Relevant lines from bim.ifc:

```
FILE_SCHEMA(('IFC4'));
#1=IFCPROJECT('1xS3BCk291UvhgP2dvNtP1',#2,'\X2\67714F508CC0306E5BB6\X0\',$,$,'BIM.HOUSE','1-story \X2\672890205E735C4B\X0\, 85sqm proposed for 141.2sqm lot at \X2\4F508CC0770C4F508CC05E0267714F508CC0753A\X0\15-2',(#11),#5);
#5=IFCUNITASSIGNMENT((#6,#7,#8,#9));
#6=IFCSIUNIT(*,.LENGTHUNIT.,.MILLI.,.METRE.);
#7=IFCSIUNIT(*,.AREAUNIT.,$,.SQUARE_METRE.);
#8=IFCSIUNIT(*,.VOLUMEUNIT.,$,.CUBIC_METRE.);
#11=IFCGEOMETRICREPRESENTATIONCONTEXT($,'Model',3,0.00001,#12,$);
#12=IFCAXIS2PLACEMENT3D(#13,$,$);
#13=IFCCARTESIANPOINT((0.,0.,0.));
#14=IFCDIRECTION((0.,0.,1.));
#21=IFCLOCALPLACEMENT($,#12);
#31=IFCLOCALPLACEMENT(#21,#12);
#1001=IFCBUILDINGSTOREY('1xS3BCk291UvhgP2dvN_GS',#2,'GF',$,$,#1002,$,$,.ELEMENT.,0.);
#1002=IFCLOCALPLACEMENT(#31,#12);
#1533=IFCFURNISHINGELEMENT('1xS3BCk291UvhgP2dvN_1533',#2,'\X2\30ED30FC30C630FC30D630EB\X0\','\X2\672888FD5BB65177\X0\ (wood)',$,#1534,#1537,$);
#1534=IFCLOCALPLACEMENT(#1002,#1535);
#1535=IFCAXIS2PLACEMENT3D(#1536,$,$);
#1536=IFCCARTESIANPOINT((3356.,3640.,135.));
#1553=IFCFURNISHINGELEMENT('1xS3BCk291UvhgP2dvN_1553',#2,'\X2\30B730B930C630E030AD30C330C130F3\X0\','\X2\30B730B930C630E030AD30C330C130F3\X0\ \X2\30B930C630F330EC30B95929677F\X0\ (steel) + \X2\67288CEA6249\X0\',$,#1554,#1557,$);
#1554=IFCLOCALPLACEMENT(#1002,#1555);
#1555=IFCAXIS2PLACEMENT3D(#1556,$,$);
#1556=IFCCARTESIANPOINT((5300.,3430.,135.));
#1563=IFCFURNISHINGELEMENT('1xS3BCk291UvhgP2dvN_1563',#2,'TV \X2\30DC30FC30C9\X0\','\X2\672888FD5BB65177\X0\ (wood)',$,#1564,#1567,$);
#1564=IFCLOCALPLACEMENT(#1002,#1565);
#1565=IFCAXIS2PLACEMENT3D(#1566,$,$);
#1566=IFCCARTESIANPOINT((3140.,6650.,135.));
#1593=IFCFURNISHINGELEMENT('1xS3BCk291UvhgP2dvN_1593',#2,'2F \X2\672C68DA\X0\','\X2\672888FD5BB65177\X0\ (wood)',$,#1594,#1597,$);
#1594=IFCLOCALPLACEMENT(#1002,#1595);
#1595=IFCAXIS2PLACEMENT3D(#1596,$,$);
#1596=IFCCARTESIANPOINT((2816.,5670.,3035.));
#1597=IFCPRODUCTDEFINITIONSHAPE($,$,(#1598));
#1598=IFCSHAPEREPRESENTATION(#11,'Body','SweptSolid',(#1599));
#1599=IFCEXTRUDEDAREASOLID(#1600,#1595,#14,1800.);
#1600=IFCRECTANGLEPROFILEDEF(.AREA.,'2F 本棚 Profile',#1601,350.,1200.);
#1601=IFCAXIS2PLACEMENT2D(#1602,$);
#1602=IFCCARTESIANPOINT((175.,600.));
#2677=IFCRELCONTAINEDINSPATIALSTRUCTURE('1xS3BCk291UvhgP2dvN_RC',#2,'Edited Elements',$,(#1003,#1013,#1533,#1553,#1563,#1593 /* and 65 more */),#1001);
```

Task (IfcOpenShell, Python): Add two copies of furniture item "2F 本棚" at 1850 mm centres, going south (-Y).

```python
import numpy as np
import ifcopenshell
import ifcopenshell.api.geometry
import ifcopenshell.api.root
import ifcopenshell.util.element
import ifcopenshell.util.placement

model = ifcopenshell.open("bim.ifc")


def reuse_history(source, copy):
    """copy_class also copies each property set's owner history, people and application; keep the originals."""
    for rel in copy.IsDefinedBy:
        if rel.is_a("IfcRelDefinesByProperties") and (history := rel.RelatingPropertyDefinition.OwnerHistory):
            rel.RelatingPropertyDefinition.OwnerHistory = source.OwnerHistory
            ifcopenshell.util.element.remove_deep2(model, history)


source = model.by_guid("1xS3BCk291UvhgP2dvN_1593")
base = ifcopenshell.util.placement.get_local_placement(source.ObjectPlacement)
step = np.array([0.0, -1.0, 0.0]) * 1850.0

for i in range(1, 3):
    copy = ifcopenshell.api.root.copy_class(model, product=source)
    copy.Representation = ifcopenshell.util.element.copy_deep(
        model, source.Representation, exclude=["IfcGeometricRepresentationContext", "IfcRepresentationMap"]
    )
    reuse_history(source, copy)
    matrix = base.copy()
    matrix[:3, 3] += i * step
    print("added at", matrix[:3, 3].round(3) + 0.0)
    ifcopenshell.api.geometry.edit_object_placement(model, product=copy, matrix=matrix, is_si=False)

model.write("bim_edited.ifc")
```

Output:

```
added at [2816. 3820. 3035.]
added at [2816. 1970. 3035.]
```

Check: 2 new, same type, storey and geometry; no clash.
